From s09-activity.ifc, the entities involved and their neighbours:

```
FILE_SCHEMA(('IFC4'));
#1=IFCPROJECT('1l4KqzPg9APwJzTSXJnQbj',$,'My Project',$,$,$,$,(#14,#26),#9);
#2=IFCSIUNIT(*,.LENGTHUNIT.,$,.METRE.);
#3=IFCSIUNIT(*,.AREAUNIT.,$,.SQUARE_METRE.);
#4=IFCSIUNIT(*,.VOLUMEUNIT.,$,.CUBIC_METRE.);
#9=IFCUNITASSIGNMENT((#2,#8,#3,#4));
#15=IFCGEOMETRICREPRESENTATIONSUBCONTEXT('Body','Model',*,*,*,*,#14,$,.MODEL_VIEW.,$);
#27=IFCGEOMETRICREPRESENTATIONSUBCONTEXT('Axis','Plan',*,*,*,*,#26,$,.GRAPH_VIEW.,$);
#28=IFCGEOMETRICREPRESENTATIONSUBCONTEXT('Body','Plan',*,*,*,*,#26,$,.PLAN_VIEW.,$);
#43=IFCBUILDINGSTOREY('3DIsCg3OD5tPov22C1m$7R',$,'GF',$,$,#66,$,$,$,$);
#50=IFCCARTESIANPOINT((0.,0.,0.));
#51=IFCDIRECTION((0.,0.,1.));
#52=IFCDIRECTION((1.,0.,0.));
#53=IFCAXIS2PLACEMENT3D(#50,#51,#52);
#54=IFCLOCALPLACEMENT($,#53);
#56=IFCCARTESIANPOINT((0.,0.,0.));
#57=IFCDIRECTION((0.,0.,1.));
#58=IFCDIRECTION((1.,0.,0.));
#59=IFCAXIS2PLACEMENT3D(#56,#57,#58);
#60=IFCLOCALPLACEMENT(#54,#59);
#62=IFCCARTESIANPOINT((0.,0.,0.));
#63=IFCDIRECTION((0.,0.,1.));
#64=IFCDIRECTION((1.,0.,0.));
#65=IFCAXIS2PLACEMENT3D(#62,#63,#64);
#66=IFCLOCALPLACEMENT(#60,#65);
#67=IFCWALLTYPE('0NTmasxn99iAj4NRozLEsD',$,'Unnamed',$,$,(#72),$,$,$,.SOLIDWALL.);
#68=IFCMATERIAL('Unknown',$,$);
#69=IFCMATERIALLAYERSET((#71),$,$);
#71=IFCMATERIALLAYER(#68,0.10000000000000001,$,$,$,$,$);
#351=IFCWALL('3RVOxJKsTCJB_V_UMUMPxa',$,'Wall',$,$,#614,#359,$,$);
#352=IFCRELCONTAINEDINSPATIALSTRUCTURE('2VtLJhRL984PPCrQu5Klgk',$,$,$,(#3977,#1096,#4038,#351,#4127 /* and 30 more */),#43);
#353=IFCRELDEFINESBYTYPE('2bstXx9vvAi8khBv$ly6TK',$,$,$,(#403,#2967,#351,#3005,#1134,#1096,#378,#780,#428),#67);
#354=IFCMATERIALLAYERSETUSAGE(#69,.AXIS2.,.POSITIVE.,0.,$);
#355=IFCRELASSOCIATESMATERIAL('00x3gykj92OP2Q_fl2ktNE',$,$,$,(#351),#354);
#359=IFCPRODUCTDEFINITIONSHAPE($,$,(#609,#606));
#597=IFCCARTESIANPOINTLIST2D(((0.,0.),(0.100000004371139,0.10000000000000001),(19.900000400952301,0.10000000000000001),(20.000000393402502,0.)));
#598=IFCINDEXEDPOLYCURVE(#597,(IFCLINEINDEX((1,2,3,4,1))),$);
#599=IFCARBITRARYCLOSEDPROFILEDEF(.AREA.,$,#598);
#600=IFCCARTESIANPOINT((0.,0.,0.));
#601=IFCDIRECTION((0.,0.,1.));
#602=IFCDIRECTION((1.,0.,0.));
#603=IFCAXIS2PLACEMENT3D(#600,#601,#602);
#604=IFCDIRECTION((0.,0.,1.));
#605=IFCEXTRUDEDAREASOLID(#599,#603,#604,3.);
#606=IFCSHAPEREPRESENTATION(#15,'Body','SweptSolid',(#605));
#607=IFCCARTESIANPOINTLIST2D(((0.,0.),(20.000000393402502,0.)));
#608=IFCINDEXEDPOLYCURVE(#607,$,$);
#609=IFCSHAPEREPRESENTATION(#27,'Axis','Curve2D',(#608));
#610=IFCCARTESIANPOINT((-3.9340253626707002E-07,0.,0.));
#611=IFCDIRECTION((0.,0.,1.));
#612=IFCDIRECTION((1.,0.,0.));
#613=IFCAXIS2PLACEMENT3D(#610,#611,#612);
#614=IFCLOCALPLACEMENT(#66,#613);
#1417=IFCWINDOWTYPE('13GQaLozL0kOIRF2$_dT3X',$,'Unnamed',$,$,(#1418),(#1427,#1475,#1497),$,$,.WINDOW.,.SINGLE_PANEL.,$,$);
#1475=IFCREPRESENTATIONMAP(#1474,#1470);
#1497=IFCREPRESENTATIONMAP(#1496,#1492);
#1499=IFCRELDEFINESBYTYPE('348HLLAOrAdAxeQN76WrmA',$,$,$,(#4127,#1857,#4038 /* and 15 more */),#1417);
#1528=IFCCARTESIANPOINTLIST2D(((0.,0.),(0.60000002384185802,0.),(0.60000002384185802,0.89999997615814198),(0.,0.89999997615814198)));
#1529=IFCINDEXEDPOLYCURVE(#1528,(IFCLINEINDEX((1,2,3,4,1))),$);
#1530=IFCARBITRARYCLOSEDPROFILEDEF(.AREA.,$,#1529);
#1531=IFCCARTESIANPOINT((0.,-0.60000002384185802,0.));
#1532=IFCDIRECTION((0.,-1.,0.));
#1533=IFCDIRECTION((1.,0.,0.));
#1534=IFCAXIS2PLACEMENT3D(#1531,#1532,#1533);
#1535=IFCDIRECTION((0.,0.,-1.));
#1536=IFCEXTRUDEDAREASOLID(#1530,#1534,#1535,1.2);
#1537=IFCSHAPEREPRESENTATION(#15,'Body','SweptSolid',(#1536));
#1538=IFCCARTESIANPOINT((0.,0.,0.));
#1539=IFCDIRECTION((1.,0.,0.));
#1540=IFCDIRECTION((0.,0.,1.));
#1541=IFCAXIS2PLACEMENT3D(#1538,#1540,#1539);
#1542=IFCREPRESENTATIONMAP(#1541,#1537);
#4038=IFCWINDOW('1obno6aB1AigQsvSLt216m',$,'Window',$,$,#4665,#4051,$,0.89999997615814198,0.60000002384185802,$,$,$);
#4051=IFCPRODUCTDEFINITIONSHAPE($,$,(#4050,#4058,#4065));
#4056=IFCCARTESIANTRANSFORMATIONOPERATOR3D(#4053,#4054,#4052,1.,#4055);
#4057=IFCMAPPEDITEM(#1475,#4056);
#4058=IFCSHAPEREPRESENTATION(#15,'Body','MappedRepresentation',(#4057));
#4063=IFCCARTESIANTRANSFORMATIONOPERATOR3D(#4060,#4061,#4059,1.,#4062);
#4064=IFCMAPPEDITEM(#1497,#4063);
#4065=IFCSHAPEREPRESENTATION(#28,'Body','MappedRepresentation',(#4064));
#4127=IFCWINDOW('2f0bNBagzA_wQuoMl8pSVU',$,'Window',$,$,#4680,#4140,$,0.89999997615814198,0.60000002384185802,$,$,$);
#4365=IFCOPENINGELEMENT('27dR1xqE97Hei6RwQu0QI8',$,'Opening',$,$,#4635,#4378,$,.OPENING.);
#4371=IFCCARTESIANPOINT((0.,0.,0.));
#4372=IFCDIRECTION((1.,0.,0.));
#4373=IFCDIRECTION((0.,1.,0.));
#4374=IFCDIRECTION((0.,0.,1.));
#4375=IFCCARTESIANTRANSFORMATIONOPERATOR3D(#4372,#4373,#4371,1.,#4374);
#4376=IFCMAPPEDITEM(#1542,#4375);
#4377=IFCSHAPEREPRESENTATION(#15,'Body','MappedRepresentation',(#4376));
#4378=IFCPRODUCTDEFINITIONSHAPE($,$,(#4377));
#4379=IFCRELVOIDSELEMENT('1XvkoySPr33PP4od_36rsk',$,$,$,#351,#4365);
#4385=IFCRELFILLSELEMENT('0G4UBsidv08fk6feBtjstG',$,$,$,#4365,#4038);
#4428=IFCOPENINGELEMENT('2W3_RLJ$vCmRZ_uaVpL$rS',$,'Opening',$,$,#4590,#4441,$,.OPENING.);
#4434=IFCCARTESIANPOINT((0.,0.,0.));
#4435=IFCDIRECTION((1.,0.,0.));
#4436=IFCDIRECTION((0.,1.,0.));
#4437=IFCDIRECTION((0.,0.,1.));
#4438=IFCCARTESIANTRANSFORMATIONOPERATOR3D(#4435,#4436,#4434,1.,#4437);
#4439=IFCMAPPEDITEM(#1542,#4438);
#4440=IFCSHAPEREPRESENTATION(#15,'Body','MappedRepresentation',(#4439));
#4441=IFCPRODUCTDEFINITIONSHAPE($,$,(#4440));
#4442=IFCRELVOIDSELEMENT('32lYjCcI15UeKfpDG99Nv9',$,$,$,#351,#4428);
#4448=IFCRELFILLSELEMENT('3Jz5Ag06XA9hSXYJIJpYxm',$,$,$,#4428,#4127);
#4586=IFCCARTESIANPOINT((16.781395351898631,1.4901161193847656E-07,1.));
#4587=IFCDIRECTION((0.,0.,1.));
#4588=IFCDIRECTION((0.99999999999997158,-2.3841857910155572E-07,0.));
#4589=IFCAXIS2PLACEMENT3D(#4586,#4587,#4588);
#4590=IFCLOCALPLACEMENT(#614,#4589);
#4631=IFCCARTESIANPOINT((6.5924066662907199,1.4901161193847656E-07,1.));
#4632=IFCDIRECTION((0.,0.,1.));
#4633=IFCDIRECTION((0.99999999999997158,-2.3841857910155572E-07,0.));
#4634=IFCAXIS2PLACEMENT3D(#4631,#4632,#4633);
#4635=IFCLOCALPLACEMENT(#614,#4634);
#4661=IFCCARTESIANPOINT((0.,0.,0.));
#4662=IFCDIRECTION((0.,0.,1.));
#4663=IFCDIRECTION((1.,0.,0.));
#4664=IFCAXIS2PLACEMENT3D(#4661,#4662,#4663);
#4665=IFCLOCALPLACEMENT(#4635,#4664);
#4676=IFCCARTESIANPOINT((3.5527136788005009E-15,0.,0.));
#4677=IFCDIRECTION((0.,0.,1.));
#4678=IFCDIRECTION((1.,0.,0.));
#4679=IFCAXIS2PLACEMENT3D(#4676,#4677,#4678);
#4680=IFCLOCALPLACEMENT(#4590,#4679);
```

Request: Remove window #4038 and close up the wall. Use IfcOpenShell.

```python
import ifcopenshell
import ifcopenshell.api.feature
import ifcopenshell.api.root
import ifcopenshell.geom
import ifcopenshell.util.shape

model = ifcopenshell.open("s09-activity.ifc")
settings = ifcopenshell.geom.settings()


def volume(element):
    """Net volume in cubic metres, openings subtracted."""
    shape = ifcopenshell.geom.create_shape(settings, element)
    return ifcopenshell.util.shape.get_volume(shape.geometry)


window = model.by_guid("1obno6aB1AigQsvSLt216m")
opening = window.FillsVoids[0].RelatingOpeningElement
wall = opening.VoidsElements[0].RelatingBuildingElement
before = volume(wall)

ifcopenshell.api.root.remove_product(model, product=window)
ifcopenshell.api.feature.remove_feature(model, feature=opening)

after = volume(wall)

print(f"wall volume {before:.3f} -> {after:.3f} m3")

model.write("s09-activity_v2.ifc")
```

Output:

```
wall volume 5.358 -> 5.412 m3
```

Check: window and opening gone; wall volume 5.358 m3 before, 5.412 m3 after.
